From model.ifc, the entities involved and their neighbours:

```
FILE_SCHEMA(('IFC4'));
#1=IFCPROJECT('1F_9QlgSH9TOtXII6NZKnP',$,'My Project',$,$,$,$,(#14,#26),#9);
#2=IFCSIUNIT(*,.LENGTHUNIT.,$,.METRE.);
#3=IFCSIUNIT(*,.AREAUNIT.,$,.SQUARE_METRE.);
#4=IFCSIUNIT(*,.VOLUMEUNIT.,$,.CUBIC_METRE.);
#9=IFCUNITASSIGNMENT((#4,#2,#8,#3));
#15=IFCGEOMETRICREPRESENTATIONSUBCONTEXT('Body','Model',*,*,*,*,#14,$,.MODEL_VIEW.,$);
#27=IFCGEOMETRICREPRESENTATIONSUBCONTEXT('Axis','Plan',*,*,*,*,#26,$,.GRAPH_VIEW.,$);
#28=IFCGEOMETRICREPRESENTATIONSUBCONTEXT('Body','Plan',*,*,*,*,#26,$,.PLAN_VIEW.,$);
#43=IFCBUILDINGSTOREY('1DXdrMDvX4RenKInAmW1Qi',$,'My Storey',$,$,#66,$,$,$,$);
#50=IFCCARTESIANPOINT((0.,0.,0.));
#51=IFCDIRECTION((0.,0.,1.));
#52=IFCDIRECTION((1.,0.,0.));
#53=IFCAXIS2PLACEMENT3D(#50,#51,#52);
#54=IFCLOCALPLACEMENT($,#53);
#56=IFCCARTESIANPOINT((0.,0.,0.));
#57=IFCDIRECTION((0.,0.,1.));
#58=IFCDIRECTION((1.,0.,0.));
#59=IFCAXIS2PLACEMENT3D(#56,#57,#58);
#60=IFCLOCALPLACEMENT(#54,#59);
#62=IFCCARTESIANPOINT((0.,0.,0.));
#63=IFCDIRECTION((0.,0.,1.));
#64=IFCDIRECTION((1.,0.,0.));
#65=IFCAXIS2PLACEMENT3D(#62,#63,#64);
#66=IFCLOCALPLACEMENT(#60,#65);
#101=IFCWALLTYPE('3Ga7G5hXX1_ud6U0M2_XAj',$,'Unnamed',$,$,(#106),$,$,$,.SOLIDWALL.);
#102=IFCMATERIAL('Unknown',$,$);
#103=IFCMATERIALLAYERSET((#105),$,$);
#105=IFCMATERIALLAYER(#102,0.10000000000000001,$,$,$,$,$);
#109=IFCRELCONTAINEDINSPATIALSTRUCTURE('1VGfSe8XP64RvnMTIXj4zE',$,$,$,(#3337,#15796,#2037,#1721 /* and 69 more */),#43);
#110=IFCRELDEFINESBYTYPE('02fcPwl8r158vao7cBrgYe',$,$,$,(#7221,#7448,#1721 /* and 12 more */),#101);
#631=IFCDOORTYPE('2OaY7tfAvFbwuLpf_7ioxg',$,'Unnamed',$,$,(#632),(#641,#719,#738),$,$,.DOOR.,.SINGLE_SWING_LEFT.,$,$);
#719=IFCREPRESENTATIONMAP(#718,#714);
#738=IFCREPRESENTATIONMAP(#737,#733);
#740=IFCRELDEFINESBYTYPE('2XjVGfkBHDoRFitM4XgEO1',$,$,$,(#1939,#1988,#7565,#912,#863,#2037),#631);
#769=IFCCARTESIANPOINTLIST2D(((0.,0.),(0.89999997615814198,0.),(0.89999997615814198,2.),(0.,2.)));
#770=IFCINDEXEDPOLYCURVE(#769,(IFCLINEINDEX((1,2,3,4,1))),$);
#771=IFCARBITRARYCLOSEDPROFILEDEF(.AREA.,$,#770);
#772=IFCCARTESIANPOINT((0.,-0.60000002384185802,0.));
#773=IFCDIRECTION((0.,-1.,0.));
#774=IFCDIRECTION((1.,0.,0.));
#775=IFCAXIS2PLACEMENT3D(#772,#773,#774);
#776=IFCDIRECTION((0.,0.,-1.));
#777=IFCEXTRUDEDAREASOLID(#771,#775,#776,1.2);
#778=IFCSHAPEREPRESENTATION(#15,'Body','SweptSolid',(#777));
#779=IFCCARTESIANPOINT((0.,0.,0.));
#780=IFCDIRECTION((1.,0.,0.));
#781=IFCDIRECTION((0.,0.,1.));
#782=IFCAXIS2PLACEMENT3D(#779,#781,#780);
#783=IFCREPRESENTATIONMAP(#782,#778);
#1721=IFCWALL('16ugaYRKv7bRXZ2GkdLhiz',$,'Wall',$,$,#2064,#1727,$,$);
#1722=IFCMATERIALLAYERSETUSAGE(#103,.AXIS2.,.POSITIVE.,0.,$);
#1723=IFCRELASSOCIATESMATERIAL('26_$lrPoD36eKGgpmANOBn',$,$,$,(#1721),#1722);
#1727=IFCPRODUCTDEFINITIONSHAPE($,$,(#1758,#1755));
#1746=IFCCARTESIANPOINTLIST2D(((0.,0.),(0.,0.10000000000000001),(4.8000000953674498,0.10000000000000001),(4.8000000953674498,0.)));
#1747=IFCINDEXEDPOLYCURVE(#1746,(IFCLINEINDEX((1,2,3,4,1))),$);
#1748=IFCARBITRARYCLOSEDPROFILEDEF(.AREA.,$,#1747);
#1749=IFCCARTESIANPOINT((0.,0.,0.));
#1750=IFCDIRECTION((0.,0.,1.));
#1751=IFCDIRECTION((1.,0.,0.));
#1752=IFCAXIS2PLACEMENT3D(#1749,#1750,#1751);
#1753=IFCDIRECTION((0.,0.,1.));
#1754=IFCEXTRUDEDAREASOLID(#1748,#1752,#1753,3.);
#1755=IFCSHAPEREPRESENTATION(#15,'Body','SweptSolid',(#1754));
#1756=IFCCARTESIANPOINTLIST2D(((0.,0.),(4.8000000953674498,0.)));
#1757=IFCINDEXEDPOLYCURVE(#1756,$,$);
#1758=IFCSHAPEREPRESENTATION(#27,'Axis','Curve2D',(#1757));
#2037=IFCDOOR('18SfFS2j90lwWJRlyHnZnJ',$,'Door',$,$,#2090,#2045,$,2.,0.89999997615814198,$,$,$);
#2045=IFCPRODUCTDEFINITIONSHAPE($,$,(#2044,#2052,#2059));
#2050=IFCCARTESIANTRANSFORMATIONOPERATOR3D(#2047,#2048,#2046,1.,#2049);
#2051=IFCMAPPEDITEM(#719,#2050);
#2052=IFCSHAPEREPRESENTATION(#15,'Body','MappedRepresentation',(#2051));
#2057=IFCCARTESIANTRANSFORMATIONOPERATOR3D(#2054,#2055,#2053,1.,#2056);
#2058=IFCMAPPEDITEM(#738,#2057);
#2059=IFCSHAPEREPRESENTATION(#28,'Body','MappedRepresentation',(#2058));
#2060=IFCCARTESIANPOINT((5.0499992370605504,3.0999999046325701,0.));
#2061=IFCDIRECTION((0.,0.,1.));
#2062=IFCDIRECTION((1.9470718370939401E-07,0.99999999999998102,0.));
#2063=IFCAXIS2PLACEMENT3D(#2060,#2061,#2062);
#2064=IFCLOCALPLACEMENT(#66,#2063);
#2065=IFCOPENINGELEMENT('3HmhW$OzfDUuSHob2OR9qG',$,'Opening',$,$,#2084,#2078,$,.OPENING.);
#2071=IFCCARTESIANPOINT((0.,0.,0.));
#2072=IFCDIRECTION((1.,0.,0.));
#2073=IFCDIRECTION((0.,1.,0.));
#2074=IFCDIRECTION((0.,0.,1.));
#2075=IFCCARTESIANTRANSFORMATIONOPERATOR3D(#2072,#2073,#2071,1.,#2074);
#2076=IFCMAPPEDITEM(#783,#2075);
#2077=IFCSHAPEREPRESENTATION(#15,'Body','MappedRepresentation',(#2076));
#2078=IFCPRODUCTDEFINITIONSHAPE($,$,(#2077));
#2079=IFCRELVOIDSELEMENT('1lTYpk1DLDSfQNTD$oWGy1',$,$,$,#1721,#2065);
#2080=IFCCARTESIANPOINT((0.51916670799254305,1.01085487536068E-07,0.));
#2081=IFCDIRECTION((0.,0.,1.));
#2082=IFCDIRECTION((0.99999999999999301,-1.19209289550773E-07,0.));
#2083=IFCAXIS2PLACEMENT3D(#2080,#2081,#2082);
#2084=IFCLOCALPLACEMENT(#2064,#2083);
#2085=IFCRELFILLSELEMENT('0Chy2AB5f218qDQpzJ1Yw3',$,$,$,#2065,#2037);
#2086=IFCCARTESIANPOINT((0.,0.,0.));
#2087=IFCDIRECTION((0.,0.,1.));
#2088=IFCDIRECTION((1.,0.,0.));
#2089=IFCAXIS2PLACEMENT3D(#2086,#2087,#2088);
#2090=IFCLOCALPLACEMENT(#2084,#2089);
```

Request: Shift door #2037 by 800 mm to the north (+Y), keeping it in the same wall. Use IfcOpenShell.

```python
import ifcopenshell
import ifcopenshell.api.geometry
import ifcopenshell.util.placement

model = ifcopenshell.open("model.ifc")

door = model.by_guid("18SfFS2j90lwWJRlyHnZnJ")
opening = door.FillsVoids[0].RelatingOpeningElement
wall = opening.VoidsElements[0].RelatingBuildingElement

wall_matrix = ifcopenshell.util.placement.get_local_placement(wall.ObjectPlacement)
shift = wall_matrix[:3, 0] * 0.8
before = ifcopenshell.util.placement.get_local_placement(door.ObjectPlacement)[:3, 3].copy()

# The door is placed relative to its opening, so it follows when the opening moves.
matrix = ifcopenshell.util.placement.get_local_placement(opening.ObjectPlacement)
matrix[:3, 3] += shift
ifcopenshell.api.geometry.edit_object_placement(
    model, product=opening, matrix=matrix, is_si=False, should_transform_children=True
)

after = ifcopenshell.util.placement.get_local_placement(door.ObjectPlacement)[:3, 3]
print("door moved by", (after - before).round(3) + 0.0)

model.write("model_rev.ifc")
```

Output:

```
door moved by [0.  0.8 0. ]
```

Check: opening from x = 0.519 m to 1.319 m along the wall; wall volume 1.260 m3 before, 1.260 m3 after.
